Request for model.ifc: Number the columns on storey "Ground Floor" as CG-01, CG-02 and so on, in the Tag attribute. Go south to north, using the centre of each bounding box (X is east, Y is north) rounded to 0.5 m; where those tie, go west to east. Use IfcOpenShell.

First a look at what the model holds.

```python
import ifcopenshell
import ifcopenshell.util.element
import ifcopenshell.util.placement

model = ifcopenshell.open("model.ifc")
print(model.schema)
storey = next(s for s in model.by_type("IfcBuildingStorey") if s.Name == "Ground Floor")
columns = [e for e in ifcopenshell.util.element.get_decomposition(storey) if e.is_a("IfcColumn")]
for e in sorted(columns, key=lambda e: e.id()):
    origin = ifcopenshell.util.placement.get_local_placement(e.ObjectPlacement)[:3, 3]
    print(e.id(), e.Tag, e.Name, origin.round(2) + 0.0, sep=" | ")
```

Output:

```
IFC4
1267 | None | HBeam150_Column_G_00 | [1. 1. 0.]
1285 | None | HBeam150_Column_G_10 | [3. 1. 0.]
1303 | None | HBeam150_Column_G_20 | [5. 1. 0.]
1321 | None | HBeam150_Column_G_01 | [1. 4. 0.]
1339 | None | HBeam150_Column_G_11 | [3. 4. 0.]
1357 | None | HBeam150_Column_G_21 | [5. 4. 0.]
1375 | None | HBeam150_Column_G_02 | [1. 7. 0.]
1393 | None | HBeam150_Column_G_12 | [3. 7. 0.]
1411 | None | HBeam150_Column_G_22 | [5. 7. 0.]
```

```python
import ifcopenshell
import ifcopenshell.geom
import ifcopenshell.util.element
import ifcopenshell.util.shape

model = ifcopenshell.open("model.ifc")
settings = ifcopenshell.geom.settings()
settings.set("use-world-coords", True)


def centre(element):
    shape = ifcopenshell.geom.create_shape(settings, element)
    return ifcopenshell.util.shape.get_bbox_centroid(shape.geometry)


storey = next(s for s in model.by_type("IfcBuildingStorey") if s.Name == "Ground Floor")
columns = [e for e in ifcopenshell.util.element.get_decomposition(storey) if e.is_a("IfcColumn")]

# Insertion points can sit at a corner or the storey origin, so sort by the geometry (in metres).
centres = {e: centre(e) for e in columns}
columns.sort(key=lambda e: (round(centres[e][1] / 0.5), centres[e][0]))

for i, e in enumerate(columns, start=1):
    number = f"CG-{i:02d}"
    e.Tag = number
    print(e.id(), number)

model.write("model_edited.ifc")
```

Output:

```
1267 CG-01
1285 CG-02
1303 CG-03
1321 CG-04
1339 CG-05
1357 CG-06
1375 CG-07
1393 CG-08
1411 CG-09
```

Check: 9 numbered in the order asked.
